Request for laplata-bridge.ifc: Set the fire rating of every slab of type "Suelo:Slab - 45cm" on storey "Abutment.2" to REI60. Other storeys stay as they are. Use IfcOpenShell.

First a look at what the model holds.

```python
import ifcopenshell
import ifcopenshell.util.element

model = ifcopenshell.open("laplata-bridge.ifc")
print(model.schema)
storey = next(s for s in model.by_type("IfcBuildingStorey") if s.Name == "Abutment.2")
slabs = [e for e in ifcopenshell.util.element.get_decomposition(storey) if e.is_a("IfcSlab")]
seen = {}
for e in slabs:
    element_type = ifcopenshell.util.element.get_type(e)
    key = (element_type.Name if element_type != e and element_type else None, ifcopenshell.util.element.get_pset(e, "Pset_SlabCommon", "FireRating"))
    seen[key] = seen.get(key, 0) + 1
for (name, value), count in sorted(seen.items(), key=str):
    print(count, "x", name, "|", value)
```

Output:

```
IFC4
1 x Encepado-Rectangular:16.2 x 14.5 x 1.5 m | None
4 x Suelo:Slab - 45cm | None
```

```python
import ifcopenshell
import ifcopenshell.api.pset
import ifcopenshell.util.element

model = ifcopenshell.open("laplata-bridge.ifc")

storey = next(s for s in model.by_type("IfcBuildingStorey") if s.Name == "Abutment.2")
slabs = [e for e in ifcopenshell.util.element.get_decomposition(storey) if e.is_a("IfcSlab")]

count = 0
for e in slabs:
    element_type = ifcopenshell.util.element.get_type(e)
    if element_type in (None, e) or element_type.Name != "Suelo:Slab - 45cm":
        continue
    # add_pset returns the element's existing set when there is one.
    pset = ifcopenshell.api.pset.add_pset(model, product=e, name="Pset_SlabCommon")
    ifcopenshell.api.pset.edit_pset(model, pset=pset, properties={"FireRating": "REI60"})
    count += 1

print(count, "slabs updated")

model.write("laplata-bridge_v2.ifc")
```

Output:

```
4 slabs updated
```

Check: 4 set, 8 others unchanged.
